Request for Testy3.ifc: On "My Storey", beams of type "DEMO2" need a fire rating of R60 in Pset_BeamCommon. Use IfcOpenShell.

First a look at what the model holds.

```python
import ifcopenshell
import ifcopenshell.util.element

model = ifcopenshell.open("Testy3.ifc")
print(model.schema)
storey = next(s for s in model.by_type("IfcBuildingStorey") if s.Name == "My Storey")
beams = [e for e in ifcopenshell.util.element.get_decomposition(storey) if e.is_a("IfcBeam")]
seen = {}
for e in beams:
    element_type = ifcopenshell.util.element.get_type(e)
    key = (element_type.Name if element_type != e and element_type else None, ifcopenshell.util.element.get_pset(e, "Pset_BeamCommon", "FireRating"))
    seen[key] = seen.get(key, 0) + 1
for (name, value), count in sorted(seen.items(), key=str):
    print(count, "x", name, "|", value)
```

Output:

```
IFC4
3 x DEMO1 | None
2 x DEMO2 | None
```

```python
import ifcopenshell
import ifcopenshell.api.pset
import ifcopenshell.util.element

model = ifcopenshell.open("Testy3.ifc")

storey = next(s for s in model.by_type("IfcBuildingStorey") if s.Name == "My Storey")
beams = [e for e in ifcopenshell.util.element.get_decomposition(storey) if e.is_a("IfcBeam")]

count = 0
for e in beams:
    element_type = ifcopenshell.util.element.get_type(e)
    if element_type in (None, e) or element_type.Name != "DEMO2":
        continue
    # add_pset returns the element's existing set when there is one.
    pset = ifcopenshell.api.pset.add_pset(model, product=e, name="Pset_BeamCommon")
    ifcopenshell.api.pset.edit_pset(model, pset=pset, properties={"FireRating": "R60"})
    count += 1

print(count, "beams updated")

model.write("Testy3-out.ifc")
```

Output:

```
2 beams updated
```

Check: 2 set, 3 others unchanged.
